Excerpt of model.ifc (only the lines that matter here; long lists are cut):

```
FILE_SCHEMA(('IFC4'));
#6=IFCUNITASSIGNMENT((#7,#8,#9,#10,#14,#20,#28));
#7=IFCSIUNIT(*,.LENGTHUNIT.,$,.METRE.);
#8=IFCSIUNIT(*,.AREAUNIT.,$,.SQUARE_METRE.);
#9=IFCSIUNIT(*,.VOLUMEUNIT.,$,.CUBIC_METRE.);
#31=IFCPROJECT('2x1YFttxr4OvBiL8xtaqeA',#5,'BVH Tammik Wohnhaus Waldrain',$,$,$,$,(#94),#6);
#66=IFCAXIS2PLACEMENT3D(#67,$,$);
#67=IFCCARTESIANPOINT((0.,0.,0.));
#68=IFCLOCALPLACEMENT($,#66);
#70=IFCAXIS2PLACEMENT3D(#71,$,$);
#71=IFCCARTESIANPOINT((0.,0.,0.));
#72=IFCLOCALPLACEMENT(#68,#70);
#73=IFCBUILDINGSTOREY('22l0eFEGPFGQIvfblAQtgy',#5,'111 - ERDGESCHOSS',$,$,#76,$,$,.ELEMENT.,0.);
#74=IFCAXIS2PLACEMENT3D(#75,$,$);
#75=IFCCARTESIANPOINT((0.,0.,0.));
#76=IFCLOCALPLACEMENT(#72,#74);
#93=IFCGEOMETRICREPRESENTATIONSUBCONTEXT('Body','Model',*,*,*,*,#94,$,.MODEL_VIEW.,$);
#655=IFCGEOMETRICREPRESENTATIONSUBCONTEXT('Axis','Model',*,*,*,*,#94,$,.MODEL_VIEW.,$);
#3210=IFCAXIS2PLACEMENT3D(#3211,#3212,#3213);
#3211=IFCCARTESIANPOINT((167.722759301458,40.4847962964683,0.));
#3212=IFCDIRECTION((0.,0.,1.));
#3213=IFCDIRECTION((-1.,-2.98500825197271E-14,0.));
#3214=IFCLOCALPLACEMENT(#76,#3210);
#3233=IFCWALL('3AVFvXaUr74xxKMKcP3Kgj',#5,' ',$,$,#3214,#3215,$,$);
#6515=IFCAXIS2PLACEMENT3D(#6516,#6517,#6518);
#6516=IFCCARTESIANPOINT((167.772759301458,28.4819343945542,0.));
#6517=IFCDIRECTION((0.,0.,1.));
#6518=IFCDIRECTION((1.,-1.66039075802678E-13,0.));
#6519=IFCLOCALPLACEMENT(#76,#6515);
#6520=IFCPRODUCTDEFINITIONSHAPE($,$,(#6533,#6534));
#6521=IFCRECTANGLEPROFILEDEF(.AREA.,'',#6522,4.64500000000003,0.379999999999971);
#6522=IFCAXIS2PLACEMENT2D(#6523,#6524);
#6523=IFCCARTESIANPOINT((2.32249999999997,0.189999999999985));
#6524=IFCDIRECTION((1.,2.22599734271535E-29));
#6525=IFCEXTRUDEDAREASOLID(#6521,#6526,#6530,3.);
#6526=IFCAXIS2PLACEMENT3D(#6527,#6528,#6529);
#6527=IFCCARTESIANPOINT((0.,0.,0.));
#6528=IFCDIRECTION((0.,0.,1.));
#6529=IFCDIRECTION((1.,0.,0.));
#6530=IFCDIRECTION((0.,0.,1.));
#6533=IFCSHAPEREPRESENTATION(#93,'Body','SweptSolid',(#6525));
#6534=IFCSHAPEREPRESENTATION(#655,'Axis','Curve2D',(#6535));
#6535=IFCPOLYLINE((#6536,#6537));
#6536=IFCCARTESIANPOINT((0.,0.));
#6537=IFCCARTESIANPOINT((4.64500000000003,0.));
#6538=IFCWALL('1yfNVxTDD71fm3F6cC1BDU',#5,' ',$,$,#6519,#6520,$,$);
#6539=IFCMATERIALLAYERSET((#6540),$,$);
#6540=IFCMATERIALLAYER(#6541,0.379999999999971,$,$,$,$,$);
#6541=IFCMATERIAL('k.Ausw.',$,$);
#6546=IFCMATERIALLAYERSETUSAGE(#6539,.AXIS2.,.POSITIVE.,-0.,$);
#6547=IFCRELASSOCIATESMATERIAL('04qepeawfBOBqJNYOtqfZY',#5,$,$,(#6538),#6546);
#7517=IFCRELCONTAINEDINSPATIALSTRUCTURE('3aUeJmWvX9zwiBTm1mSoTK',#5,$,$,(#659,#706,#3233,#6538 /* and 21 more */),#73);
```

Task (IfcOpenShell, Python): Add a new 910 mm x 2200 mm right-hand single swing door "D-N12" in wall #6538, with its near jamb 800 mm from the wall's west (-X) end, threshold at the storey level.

```python
import numpy as np
import ifcopenshell
import ifcopenshell.api.feature
import ifcopenshell.api.geometry
import ifcopenshell.api.root
import ifcopenshell.api.spatial
import ifcopenshell.geom
import ifcopenshell.util.element
import ifcopenshell.util.placement
import ifcopenshell.util.representation
import ifcopenshell.util.shape
import ifcopenshell.util.unit

model = ifcopenshell.open("model.ifc")
unit_scale = ifcopenshell.util.unit.calculate_unit_scale(model)
settings = ifcopenshell.geom.settings()


def volume(element):
    """Net volume in cubic metres, openings subtracted."""
    shape = ifcopenshell.geom.create_shape(settings, element)
    return ifcopenshell.util.shape.get_volume(shape.geometry)


wall = model.by_guid("1yfNVxTDD71fm3F6cC1BDU")
storey = ifcopenshell.util.element.get_container(wall, ifc_class="IfcBuildingStorey")
context = ifcopenshell.util.representation.get_context(model, "Model", "Body", "MODEL_VIEW")
before = volume(wall)

width, height, from_end, sill = 0.91, 2.2, 0.8, 0.0  # metres

# The wall runs along its own X axis, and the end named is its -X end.
wall_shape = ifcopenshell.geom.create_shape(settings, wall)
x, y, z = ifcopenshell.util.shape.get_vertices(wall_shape.geometry).T
start = x.min() + from_end
face, thickness = float(y.min()), float(y.max() - y.min())
wall_matrix = ifcopenshell.util.placement.get_local_placement(wall.ObjectPlacement)
level = ifcopenshell.util.placement.get_local_placement(storey.ObjectPlacement)[2, 3]


def in_wall(x, y):
    """Placement at x, y metres in the wall's axes, at sill height."""
    matrix = wall_matrix.copy()
    matrix[:, 3] = wall_matrix @ np.array([x / unit_scale, y / unit_scale, 0.0, 1.0])
    matrix[2, 3] = level + sill / unit_scale
    return matrix


# Opening: a box that overshoots both wall faces by 50 mm.
opening = ifcopenshell.api.root.create_entity(model, ifc_class="IfcOpeningElement", predefined_type="OPENING")
box = ifcopenshell.api.geometry.add_wall_representation(
    model, context=context, length=width, height=height, thickness=thickness + 0.1
)
ifcopenshell.api.geometry.assign_representation(model, product=opening, representation=box)
ifcopenshell.api.geometry.edit_object_placement(model, product=opening, matrix=in_wall(start, face - 0.05), is_si=False)
ifcopenshell.api.feature.add_feature(model, feature=opening, element=wall)

door = ifcopenshell.api.root.create_entity(model, ifc_class="IfcDoor", name="D-N12", predefined_type="DOOR")
door.OverallWidth, door.OverallHeight = width / unit_scale, height / unit_scale
door.OperationType = "SINGLE_SWING_RIGHT"
body = ifcopenshell.api.geometry.add_door_representation(
    model,
    context=context,
    overall_width=door.OverallWidth,
    overall_height=door.OverallHeight,
    operation_type="SINGLE_SWING_RIGHT",
    lining_properties={"LiningDepth": thickness / unit_scale, "ThresholdDepth": thickness / unit_scale},
)
ifcopenshell.api.geometry.assign_representation(model, product=door, representation=body)
ifcopenshell.api.spatial.assign_container(model, products=[door], relating_structure=storey)
ifcopenshell.api.feature.add_filling(model, opening=opening, element=door)

# The lining spans the wall, so the door starts at the wall face.
ifcopenshell.api.geometry.edit_object_placement(model, product=door, matrix=in_wall(start, face), is_si=False)

after = volume(wall)

print(f"wall volume {before:.3f} -> {after:.3f} m3")

model.write("model_v2.ifc")
```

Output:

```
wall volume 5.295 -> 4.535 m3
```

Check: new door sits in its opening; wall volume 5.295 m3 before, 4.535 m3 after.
